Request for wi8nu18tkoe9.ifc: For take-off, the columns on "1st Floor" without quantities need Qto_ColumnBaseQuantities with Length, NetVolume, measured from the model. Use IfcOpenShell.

First a look at what the model holds.

```python
import ifcopenshell
import ifcopenshell.util.element
import ifcopenshell.util.unit

model = ifcopenshell.open("wi8nu18tkoe9.ifc")
print(model.schema)
for unit_type in ("LENGTHUNIT", "AREAUNIT", "VOLUMEUNIT"):
    print(unit_type, ifcopenshell.util.unit.calculate_unit_scale(model, unit_type))
storey = next(s for s in model.by_type("IfcBuildingStorey") if s.Name == "1st Floor")
columns = [e for e in ifcopenshell.util.element.get_decomposition(storey) if e.is_a("IfcColumn")]
for e in sorted(columns, key=lambda e: e.id()):
    print(e.id(), e.is_a(), e.Name, list(ifcopenshell.util.element.get_psets(e, qtos_only=True)), sep=" | ")
```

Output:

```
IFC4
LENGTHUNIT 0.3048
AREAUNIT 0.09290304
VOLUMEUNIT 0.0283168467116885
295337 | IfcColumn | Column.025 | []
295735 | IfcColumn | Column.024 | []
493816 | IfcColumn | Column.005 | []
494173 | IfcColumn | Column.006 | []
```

```python
import ifcopenshell
import ifcopenshell.api.pset
import ifcopenshell.geom
import ifcopenshell.util.element
import ifcopenshell.util.shape
import ifcopenshell.util.unit

model = ifcopenshell.open("wi8nu18tkoe9.ifc")
unit_scale = ifcopenshell.util.unit.calculate_unit_scale(model)
volume_scale = ifcopenshell.util.unit.calculate_unit_scale(model, "VOLUMEUNIT")
settings = ifcopenshell.geom.settings()

storey = next(s for s in model.by_type("IfcBuildingStorey") if s.Name == "1st Floor")
columns = [e for e in ifcopenshell.util.element.get_decomposition(storey) if e.is_a("IfcColumn")]

for e in sorted(columns, key=lambda e: e.id()):
    if ifcopenshell.util.element.get_psets(e, qtos_only=True, should_inherit=False):
        continue
    # Geometry comes back in metres, in the element's own axes.
    shape = ifcopenshell.geom.create_shape(settings, e)
    values = {
        "Length": ifcopenshell.util.shape.get_z(shape.geometry) / unit_scale,
        "NetVolume": ifcopenshell.util.shape.get_volume(shape.geometry) / volume_scale,
    }
    qto = ifcopenshell.api.pset.add_qto(model, product=e, name="Qto_ColumnBaseQuantities")
    ifcopenshell.api.pset.edit_qto(model, qto=qto, properties=values)
    print(e.id(), {k: round(v, 3) for k, v in values.items()})

model.write("wi8nu18tkoe9_v2.ifc")
```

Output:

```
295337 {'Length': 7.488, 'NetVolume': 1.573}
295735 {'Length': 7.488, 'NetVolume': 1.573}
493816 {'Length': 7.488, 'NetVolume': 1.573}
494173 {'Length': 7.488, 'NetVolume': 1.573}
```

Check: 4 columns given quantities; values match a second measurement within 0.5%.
